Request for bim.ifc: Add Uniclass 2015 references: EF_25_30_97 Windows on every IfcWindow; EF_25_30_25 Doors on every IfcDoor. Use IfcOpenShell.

First a look at what the model holds.

```python
import ifcopenshell

model = ifcopenshell.open("bim.ifc")
print(model.schema)
print("classifications:", [c.Name for c in model.by_type("IfcClassification")])
for ifc_class in ("IfcDoor", "IfcRoof", "IfcStair", "IfcWall", "IfcWindow"):
    print(ifc_class, len(model.by_type(ifc_class)))
```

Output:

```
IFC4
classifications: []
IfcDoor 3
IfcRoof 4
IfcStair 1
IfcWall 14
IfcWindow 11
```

```python
import ifcopenshell
import ifcopenshell.api.classification

model = ifcopenshell.open("bim.ifc")

system = ifcopenshell.api.classification.add_classification(model, classification="Uniclass 2015")

codes = {
    "IfcWindow": ("EF_25_30_97", "Windows"),
    "IfcDoor": ("EF_25_30_25", "Doors"),
}
for ifc_class, (code, name) in codes.items():
    products = model.by_type(ifc_class)
    ifcopenshell.api.classification.add_reference(
        model, products=products, classification=system, identification=code, name=name
    )
    print(code, len(products))

model.write("bim_updated.ifc")
```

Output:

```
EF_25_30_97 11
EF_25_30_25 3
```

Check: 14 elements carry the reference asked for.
